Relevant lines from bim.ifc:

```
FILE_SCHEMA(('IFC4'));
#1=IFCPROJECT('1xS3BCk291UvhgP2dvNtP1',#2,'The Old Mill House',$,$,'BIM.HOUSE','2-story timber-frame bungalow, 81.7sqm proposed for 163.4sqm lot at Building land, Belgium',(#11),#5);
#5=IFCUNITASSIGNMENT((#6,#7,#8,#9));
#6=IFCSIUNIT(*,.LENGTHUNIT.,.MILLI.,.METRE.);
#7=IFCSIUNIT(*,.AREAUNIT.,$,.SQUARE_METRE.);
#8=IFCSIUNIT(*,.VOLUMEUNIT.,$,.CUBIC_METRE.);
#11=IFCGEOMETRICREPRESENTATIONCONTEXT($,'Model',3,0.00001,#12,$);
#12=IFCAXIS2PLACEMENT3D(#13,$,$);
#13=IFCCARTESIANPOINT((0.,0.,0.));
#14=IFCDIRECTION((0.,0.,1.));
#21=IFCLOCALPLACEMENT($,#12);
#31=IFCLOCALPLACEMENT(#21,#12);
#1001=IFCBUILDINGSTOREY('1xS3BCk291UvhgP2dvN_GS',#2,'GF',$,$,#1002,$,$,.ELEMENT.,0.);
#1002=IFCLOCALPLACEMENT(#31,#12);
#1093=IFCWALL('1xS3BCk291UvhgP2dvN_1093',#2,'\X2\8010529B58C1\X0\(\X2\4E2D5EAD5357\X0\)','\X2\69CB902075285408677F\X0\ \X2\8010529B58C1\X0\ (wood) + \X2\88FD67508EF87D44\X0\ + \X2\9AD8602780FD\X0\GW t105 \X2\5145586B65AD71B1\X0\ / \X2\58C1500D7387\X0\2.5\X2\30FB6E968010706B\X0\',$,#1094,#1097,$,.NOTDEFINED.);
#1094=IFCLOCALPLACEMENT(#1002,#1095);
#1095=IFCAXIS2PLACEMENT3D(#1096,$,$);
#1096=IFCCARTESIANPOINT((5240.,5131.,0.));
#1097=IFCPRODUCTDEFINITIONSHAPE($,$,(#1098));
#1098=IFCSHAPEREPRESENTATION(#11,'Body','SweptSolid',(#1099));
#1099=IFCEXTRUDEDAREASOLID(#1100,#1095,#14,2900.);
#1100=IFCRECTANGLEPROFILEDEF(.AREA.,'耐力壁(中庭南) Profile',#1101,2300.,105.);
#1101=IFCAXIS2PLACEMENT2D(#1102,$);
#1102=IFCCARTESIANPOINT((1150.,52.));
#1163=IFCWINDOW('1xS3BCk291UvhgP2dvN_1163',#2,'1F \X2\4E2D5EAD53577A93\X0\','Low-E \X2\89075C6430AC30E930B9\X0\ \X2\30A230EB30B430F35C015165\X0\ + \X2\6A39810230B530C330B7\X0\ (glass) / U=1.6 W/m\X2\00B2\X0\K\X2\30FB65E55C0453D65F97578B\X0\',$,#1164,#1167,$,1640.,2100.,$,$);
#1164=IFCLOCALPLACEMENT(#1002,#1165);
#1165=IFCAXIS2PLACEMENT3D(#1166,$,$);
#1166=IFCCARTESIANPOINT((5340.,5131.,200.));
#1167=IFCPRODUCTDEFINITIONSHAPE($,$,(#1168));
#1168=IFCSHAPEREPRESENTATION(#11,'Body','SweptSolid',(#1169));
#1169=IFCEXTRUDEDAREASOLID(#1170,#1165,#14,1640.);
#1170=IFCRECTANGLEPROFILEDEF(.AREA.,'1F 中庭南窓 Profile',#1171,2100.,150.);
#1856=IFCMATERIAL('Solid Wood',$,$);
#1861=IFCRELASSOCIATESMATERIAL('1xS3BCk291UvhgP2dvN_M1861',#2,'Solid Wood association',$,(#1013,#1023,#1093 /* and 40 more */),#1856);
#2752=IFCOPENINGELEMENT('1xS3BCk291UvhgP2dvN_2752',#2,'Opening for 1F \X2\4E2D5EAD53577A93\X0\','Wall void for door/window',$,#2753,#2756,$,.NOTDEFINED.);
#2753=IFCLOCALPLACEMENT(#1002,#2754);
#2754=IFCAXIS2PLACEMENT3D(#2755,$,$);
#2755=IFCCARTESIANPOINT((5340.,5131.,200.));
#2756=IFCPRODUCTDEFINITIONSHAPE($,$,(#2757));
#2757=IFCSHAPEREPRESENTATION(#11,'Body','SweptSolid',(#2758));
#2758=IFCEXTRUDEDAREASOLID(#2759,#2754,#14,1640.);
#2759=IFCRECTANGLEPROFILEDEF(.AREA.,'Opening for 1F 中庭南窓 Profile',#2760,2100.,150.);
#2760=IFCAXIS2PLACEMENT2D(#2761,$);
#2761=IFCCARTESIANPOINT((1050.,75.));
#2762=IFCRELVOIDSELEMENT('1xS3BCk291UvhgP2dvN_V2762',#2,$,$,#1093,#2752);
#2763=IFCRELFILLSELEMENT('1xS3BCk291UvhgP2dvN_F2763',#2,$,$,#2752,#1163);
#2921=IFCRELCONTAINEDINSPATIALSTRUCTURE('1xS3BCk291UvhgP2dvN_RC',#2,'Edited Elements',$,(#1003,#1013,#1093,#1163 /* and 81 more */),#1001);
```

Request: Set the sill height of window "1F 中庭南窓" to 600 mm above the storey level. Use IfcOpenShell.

```python
import numpy as np
import ifcopenshell
import ifcopenshell.api.geometry
import ifcopenshell.geom
import ifcopenshell.util.element
import ifcopenshell.util.placement
import ifcopenshell.util.shape
import ifcopenshell.util.unit

model = ifcopenshell.open("bim.ifc")
unit_scale = ifcopenshell.util.unit.calculate_unit_scale(model)

window = model.by_id(1163)
opening = window.FillsVoids[0].RelatingOpeningElement
storey = ifcopenshell.util.element.get_container(window, ifc_class="IfcBuildingStorey")
level = ifcopenshell.util.placement.get_local_placement(storey.ObjectPlacement)[2, 3]

# The opening's origin need not be at the sill, so measure its lowest point.
shape = ifcopenshell.geom.create_shape(ifcopenshell.geom.settings(), opening)
bottom = ifcopenshell.util.shape.get_shape_bottom_elevation(shape, shape.geometry) / unit_scale
dz = level + 0.6 / unit_scale - bottom

shift = np.array([0.0, 0.0, dz])
# The window is not placed relative to its opening, so move both.
for product in (opening, window):
    matrix = ifcopenshell.util.placement.get_local_placement(product.ObjectPlacement)
    matrix[:3, 3] += shift
    ifcopenshell.api.geometry.edit_object_placement(model, product=product, matrix=matrix, is_si=False)

print(f"moved by {dz * unit_scale:+.3f} m")

model.write("bim_edited.ifc")
```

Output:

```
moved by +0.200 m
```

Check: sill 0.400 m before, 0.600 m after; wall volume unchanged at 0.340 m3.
